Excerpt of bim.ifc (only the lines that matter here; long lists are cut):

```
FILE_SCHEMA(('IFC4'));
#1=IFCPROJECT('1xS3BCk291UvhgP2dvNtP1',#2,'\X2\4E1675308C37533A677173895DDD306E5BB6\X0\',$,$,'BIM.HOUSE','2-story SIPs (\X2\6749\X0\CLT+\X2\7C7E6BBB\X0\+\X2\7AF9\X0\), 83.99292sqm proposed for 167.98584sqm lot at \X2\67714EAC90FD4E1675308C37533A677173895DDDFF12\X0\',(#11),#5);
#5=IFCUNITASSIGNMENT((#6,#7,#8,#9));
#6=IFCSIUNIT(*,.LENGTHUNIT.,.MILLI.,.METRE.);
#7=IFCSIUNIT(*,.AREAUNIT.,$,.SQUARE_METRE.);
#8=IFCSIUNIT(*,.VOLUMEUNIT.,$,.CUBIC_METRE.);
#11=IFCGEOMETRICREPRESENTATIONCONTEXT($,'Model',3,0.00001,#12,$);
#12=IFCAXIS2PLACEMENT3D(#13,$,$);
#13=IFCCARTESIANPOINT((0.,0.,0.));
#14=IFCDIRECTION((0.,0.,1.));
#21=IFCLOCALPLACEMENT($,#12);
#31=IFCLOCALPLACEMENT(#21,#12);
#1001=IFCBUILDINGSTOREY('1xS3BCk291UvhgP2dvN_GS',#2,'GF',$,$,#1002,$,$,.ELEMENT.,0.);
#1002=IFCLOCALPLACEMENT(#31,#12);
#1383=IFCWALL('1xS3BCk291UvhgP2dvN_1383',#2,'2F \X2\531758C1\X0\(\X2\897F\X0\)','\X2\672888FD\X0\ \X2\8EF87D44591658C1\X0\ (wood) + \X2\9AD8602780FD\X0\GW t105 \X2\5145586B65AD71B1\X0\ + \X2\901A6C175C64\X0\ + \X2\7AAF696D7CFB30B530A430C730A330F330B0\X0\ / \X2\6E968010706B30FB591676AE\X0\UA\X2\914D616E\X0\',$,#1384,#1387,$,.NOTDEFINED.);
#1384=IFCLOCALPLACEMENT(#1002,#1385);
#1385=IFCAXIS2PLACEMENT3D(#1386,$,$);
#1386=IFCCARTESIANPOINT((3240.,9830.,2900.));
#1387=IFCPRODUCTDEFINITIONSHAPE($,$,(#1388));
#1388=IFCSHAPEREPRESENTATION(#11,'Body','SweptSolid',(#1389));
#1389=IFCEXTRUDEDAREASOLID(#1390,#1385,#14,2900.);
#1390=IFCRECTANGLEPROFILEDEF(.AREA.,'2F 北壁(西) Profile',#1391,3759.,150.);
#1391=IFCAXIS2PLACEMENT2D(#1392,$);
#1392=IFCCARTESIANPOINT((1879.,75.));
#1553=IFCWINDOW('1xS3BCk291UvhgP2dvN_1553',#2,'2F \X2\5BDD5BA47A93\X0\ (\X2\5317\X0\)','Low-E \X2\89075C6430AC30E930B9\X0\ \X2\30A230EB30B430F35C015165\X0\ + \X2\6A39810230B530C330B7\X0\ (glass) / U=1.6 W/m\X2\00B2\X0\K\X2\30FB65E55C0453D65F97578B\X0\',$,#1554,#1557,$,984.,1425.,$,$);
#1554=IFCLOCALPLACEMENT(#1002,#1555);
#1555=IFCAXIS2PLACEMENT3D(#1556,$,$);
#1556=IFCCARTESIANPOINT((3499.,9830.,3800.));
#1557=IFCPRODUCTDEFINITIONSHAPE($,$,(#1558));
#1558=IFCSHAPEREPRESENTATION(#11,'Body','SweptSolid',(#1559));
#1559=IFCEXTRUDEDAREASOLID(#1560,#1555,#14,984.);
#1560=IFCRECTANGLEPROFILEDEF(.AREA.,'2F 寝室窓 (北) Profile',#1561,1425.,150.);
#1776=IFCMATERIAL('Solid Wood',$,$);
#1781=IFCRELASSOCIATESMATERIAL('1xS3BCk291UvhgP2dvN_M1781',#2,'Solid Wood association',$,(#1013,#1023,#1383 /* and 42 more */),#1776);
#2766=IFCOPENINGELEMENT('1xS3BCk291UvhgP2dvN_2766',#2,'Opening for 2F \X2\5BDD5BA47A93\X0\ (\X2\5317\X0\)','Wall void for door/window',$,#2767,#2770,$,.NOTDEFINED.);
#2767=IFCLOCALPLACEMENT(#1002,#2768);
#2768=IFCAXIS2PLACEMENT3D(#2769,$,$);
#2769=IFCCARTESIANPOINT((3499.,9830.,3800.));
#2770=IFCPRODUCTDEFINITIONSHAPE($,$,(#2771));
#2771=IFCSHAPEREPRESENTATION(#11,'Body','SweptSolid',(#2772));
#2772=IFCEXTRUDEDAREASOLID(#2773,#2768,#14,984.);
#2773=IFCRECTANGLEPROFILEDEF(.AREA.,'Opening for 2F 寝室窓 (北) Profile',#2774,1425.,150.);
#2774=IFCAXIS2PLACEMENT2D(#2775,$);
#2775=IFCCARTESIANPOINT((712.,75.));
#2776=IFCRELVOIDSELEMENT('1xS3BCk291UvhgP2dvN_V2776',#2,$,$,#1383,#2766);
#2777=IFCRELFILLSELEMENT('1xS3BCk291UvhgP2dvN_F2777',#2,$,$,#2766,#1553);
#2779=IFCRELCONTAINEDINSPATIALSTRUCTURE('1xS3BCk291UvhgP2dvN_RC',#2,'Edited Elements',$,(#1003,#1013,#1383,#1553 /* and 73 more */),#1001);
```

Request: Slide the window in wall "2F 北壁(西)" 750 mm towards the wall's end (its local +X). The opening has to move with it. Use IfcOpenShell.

```python
import ifcopenshell
import ifcopenshell.api.geometry
import ifcopenshell.util.placement
import ifcopenshell.util.unit

model = ifcopenshell.open("bim.ifc")
unit_scale = ifcopenshell.util.unit.calculate_unit_scale(model)

window = model.by_guid("1xS3BCk291UvhgP2dvN_1553")
opening = window.FillsVoids[0].RelatingOpeningElement
wall = opening.VoidsElements[0].RelatingBuildingElement

wall_matrix = ifcopenshell.util.placement.get_local_placement(wall.ObjectPlacement)
shift = wall_matrix[:3, 0] * 0.75 / unit_scale
before = ifcopenshell.util.placement.get_local_placement(window.ObjectPlacement)[:3, 3].copy()

# The window is not placed relative to its opening, so move both.
for product in (opening, window):
    matrix = ifcopenshell.util.placement.get_local_placement(product.ObjectPlacement)
    matrix[:3, 3] += shift
    ifcopenshell.api.geometry.edit_object_placement(model, product=product, matrix=matrix, is_si=False)

after = ifcopenshell.util.placement.get_local_placement(window.ObjectPlacement)[:3, 3]
print("window moved by", (after - before).round(3) + 0.0)

model.write("bim_rev.ifc")
```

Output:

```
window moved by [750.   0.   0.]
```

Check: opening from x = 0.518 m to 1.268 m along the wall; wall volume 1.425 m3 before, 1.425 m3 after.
